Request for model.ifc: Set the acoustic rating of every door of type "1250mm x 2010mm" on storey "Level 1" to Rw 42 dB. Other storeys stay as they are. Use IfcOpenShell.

First a look at what the model holds.

```python
import ifcopenshell
import ifcopenshell.util.element

model = ifcopenshell.open("model.ifc")
print(model.schema)
storey = next(s for s in model.by_type("IfcBuildingStorey") if s.Name == "Level 1")
doors = [e for e in ifcopenshell.util.element.get_decomposition(storey) if e.is_a("IfcDoor")]
seen = {}
for e in doors:
    element_type = ifcopenshell.util.element.get_type(e)
    key = (element_type.Name if element_type != e and element_type else None, ifcopenshell.util.element.get_pset(e, "Pset_DoorCommon", "AcousticRating"))
    seen[key] = seen.get(key, 0) + 1
for (name, value), count in sorted(seen.items(), key=str):
    print(count, "x", name, "|", value)
```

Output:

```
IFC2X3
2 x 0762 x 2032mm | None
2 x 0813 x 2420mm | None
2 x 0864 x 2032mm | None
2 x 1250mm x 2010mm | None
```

```python
import ifcopenshell
import ifcopenshell.api.pset
import ifcopenshell.util.element

model = ifcopenshell.open("model.ifc")

storey = next(s for s in model.by_type("IfcBuildingStorey") if s.Name == "Level 1")
doors = [e for e in ifcopenshell.util.element.get_decomposition(storey) if e.is_a("IfcDoor")]

count = 0
for e in doors:
    element_type = ifcopenshell.util.element.get_type(e)
    if element_type in (None, e) or element_type.Name != "1250mm x 2010mm":
        continue
    # add_pset returns the element's existing set when there is one.
    pset = ifcopenshell.api.pset.add_pset(model, product=e, name="Pset_DoorCommon")
    ifcopenshell.api.pset.edit_pset(model, pset=pset, properties={"AcousticRating": "Rw 42 dB"})
    count += 1

print(count, "doors updated")

model.write("model_v2.ifc")
```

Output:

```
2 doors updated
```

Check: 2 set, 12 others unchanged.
